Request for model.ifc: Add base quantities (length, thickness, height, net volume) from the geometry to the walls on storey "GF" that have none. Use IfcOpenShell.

First a look at what the model holds.

```python
import ifcopenshell
import ifcopenshell.util.element
import ifcopenshell.util.unit

model = ifcopenshell.open("model.ifc")
print(model.schema)
for unit_type in ("LENGTHUNIT", "AREAUNIT", "VOLUMEUNIT"):
    print(unit_type, ifcopenshell.util.unit.calculate_unit_scale(model, unit_type))
storey = next(s for s in model.by_type("IfcBuildingStorey") if s.Name == "GF")
walls = [e for e in ifcopenshell.util.element.get_decomposition(storey) if e.is_a("IfcWall")]
for e in sorted(walls, key=lambda e: e.id()):
    print(e.id(), e.is_a(), e.Name, list(ifcopenshell.util.element.get_psets(e, qtos_only=True)), sep=" | ")
```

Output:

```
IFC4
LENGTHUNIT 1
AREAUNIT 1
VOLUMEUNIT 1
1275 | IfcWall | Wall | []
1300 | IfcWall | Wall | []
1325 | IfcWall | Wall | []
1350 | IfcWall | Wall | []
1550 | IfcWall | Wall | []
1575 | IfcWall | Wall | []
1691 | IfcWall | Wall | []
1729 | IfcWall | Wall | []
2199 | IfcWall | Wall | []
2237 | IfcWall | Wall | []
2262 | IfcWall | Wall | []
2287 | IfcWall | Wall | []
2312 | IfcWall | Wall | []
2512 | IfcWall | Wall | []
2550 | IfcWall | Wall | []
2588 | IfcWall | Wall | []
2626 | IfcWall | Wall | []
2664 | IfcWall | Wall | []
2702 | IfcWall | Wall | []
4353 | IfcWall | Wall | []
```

```python
import ifcopenshell
import ifcopenshell.api.pset
import ifcopenshell.geom
import ifcopenshell.util.element
import ifcopenshell.util.shape
import ifcopenshell.util.unit

model = ifcopenshell.open("model.ifc")
unit_scale = ifcopenshell.util.unit.calculate_unit_scale(model)
volume_scale = ifcopenshell.util.unit.calculate_unit_scale(model, "VOLUMEUNIT")
settings = ifcopenshell.geom.settings()

storey = next(s for s in model.by_type("IfcBuildingStorey") if s.Name == "GF")
walls = [e for e in ifcopenshell.util.element.get_decomposition(storey) if e.is_a("IfcWall")]

for e in sorted(walls, key=lambda e: e.id()):
    if ifcopenshell.util.element.get_psets(e, qtos_only=True, should_inherit=False):
        continue
    # Geometry comes back in metres, in the element's own axes.
    shape = ifcopenshell.geom.create_shape(settings, e)
    values = {
        "Length": ifcopenshell.util.shape.get_x(shape.geometry) / unit_scale,
        "Width": ifcopenshell.util.shape.get_y(shape.geometry) / unit_scale,
        "Height": ifcopenshell.util.shape.get_z(shape.geometry) / unit_scale,
        "NetVolume": ifcopenshell.util.shape.get_volume(shape.geometry) / volume_scale,
    }
    qto = ifcopenshell.api.pset.add_qto(model, product=e, name="Qto_WallBaseQuantities")
    ifcopenshell.api.pset.edit_qto(model, qto=qto, properties=values)
    print(e.id(), {k: round(v, 3) for k, v in values.items()})

model.write("model_updated.ifc")
```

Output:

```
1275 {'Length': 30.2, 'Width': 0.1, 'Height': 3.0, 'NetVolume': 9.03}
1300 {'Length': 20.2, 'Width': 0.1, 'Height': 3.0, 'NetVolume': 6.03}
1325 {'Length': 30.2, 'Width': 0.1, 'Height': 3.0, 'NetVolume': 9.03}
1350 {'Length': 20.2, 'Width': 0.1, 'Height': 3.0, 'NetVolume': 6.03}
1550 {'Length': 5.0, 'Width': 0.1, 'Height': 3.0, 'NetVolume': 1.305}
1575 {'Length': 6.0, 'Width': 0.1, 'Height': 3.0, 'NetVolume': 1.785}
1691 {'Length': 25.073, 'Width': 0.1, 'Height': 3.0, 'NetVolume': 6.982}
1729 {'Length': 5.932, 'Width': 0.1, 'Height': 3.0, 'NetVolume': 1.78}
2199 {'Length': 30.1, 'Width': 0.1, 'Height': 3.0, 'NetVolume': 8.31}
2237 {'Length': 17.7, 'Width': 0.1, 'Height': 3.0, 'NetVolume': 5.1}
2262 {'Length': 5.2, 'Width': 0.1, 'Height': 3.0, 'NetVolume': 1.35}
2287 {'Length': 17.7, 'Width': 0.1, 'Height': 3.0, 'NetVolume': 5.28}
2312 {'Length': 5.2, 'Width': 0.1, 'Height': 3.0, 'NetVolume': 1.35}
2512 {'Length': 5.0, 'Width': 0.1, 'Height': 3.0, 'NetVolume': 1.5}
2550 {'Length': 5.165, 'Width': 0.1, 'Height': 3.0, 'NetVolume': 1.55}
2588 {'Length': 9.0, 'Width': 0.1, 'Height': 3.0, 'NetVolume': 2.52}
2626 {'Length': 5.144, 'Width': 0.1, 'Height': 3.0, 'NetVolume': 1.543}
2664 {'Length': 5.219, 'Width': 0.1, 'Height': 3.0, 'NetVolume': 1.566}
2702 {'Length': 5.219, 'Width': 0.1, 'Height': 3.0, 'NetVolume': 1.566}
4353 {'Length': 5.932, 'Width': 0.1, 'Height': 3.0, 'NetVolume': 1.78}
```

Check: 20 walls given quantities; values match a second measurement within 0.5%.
